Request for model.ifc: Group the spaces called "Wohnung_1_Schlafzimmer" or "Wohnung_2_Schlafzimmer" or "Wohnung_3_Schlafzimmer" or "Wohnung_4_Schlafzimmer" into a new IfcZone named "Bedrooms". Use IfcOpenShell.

First a look at what the model holds.

```python
import ifcopenshell

model = ifcopenshell.open("model.ifc")
print(model.schema)
seen = {}
for space in model.by_type("IfcSpace"):
    seen[space.LongName] = seen.get(space.LongName, 0) + 1
for name, count in sorted(seen.items(), key=str):
    print(count, "x", name)
print("zones:", [z.Name for z in model.by_type("IfcZone")][:20])
```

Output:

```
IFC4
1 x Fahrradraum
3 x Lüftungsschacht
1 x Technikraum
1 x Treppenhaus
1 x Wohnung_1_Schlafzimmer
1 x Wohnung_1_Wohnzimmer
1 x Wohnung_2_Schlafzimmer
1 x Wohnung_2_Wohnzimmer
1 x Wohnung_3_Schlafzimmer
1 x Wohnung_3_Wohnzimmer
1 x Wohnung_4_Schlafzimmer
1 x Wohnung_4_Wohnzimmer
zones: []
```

```python
import ifcopenshell
import ifcopenshell.api.group
import ifcopenshell.api.root

model = ifcopenshell.open("model.ifc")

names = {"Wohnung_1_Schlafzimmer", "Wohnung_2_Schlafzimmer", "Wohnung_3_Schlafzimmer", "Wohnung_4_Schlafzimmer"}
spaces = [s for s in model.by_type("IfcSpace") if s.LongName in names]

zone = ifcopenshell.api.root.create_entity(model, ifc_class="IfcZone", name="Bedrooms")
ifcopenshell.api.group.assign_group(model, products=spaces, group=zone)
print(len(spaces), "spaces in", zone.Name)

model.write("model-out.ifc")
```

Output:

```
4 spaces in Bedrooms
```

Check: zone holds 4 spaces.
